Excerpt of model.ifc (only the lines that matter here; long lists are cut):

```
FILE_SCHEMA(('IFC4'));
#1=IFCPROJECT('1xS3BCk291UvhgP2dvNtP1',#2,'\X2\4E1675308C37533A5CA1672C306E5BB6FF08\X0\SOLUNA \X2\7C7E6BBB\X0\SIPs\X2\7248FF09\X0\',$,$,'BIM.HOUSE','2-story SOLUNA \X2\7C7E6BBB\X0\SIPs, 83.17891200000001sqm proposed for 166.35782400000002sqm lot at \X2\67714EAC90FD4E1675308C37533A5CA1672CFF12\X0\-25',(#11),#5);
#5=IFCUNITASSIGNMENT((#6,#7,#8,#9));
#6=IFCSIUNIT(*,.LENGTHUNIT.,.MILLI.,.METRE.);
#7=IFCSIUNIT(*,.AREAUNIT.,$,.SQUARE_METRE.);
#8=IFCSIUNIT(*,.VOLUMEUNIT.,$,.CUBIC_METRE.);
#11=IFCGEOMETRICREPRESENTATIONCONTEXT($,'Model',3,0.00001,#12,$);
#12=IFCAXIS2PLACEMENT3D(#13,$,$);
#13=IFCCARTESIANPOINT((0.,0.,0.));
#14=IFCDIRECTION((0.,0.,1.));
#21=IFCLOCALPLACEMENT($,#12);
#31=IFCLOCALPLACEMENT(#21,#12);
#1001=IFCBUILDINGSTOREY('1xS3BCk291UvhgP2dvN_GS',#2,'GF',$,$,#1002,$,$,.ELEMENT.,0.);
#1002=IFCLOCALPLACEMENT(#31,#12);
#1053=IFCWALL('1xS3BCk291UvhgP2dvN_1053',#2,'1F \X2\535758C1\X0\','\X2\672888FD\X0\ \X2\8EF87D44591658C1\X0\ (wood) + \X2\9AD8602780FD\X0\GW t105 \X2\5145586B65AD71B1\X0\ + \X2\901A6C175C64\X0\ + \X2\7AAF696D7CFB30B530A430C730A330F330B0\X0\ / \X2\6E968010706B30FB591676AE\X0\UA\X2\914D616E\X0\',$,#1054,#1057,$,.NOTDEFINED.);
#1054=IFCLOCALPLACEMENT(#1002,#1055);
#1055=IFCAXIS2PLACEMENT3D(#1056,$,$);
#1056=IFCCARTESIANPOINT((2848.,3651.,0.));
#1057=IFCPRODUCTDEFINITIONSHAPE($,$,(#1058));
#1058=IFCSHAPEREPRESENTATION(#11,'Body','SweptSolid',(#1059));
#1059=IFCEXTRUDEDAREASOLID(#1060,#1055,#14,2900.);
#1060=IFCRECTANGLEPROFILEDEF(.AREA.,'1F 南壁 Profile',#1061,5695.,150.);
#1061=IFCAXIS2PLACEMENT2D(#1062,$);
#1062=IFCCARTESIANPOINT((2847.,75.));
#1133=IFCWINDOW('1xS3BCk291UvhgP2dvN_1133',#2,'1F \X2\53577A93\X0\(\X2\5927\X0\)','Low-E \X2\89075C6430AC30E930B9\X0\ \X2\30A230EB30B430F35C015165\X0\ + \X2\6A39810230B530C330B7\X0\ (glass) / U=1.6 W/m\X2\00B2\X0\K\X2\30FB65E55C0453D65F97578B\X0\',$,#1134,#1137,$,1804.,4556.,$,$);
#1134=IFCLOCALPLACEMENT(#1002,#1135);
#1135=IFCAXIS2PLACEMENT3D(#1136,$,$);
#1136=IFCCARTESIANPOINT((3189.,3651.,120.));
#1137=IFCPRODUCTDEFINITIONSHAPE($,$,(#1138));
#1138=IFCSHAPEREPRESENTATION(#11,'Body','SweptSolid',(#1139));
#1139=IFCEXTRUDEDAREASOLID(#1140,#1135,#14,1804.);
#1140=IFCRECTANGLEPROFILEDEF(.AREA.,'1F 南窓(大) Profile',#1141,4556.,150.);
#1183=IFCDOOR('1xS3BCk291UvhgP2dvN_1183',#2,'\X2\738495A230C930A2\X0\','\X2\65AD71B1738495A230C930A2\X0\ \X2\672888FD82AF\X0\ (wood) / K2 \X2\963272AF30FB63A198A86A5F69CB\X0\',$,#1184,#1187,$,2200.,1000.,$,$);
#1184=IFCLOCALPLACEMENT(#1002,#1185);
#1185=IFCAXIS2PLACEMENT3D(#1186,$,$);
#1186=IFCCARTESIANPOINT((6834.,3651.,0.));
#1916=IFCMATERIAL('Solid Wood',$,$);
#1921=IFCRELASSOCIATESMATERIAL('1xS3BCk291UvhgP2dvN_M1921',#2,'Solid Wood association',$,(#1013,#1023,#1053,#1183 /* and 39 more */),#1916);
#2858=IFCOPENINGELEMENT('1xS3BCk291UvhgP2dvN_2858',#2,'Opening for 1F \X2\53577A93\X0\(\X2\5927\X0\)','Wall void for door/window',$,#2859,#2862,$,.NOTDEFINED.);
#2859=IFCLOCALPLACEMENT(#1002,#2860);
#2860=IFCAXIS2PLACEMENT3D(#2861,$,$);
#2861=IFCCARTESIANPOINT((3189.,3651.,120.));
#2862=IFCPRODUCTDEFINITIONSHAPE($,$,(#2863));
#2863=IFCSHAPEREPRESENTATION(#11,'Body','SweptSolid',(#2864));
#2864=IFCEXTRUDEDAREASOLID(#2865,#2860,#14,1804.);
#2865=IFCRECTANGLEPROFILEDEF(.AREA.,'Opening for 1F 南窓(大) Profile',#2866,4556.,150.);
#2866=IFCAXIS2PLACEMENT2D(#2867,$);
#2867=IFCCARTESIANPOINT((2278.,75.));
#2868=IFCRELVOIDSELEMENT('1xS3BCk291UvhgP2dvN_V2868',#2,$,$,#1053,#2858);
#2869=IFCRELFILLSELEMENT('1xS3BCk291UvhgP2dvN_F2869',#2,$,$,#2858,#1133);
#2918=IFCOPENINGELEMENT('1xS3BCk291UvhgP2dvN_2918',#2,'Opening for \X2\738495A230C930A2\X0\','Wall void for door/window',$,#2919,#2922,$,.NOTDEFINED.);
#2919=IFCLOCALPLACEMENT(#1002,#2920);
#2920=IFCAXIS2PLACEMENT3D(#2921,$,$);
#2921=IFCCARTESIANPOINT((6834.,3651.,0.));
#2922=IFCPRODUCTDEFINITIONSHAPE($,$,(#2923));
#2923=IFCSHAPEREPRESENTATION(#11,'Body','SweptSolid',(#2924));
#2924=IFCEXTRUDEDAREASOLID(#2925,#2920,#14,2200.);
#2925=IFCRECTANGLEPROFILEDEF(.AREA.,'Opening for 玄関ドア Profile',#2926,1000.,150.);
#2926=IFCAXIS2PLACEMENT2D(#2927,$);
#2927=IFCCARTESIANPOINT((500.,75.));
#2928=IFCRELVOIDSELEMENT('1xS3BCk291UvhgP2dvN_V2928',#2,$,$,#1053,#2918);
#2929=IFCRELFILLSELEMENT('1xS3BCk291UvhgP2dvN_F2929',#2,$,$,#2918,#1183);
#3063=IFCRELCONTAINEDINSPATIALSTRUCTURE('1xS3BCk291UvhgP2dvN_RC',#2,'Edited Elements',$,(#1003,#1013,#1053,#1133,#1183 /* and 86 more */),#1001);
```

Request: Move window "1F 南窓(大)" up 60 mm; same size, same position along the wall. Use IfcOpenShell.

```python
import numpy as np
import ifcopenshell
import ifcopenshell.api.geometry
import ifcopenshell.util.placement
import ifcopenshell.util.unit

model = ifcopenshell.open("model.ifc")
unit_scale = ifcopenshell.util.unit.calculate_unit_scale(model)

window = model.by_guid("1xS3BCk291UvhgP2dvN_1133")
opening = window.FillsVoids[0].RelatingOpeningElement
dz = 60.0

shift = np.array([0.0, 0.0, dz])
# The window is not placed relative to its opening, so move both.
for product in (opening, window):
    matrix = ifcopenshell.util.placement.get_local_placement(product.ObjectPlacement)
    matrix[:3, 3] += shift
    ifcopenshell.api.geometry.edit_object_placement(model, product=product, matrix=matrix, is_si=False)

print(f"moved by {dz * unit_scale:+.3f} m")

model.write("model-out.ifc")
```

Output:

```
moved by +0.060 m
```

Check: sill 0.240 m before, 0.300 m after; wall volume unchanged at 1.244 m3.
